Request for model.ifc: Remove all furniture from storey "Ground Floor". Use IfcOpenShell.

First a look at what the model holds.

```python
import ifcopenshell
import ifcopenshell.util.element

model = ifcopenshell.open("model.ifc")
print(model.schema)
storey = next(s for s in model.by_type("IfcBuildingStorey") if s.Name == "Ground Floor")
furniture = [e for e in ifcopenshell.util.element.get_decomposition(storey) if e.is_a("IfcFurnishingElement")]
seen = {}
for e in furniture:
    element_type = ifcopenshell.util.element.get_type(e)
    name = element_type.Name if element_type not in (None, e) else None
    seen[name] = seen.get(name, 0) + 1
for name, count in sorted(seen.items(), key=str):
    print(count, "x", name)
```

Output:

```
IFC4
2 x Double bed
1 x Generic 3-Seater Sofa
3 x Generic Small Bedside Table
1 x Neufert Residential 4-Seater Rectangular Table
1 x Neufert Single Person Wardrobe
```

```python
import ifcopenshell
import ifcopenshell.api.root
import ifcopenshell.util.element

model = ifcopenshell.open("model.ifc")

storey = next(s for s in model.by_type("IfcBuildingStorey") if s.Name == "Ground Floor")
furniture = [e for e in ifcopenshell.util.element.get_decomposition(storey) if e.is_a("IfcFurnishingElement")]

for e in furniture:
    ifcopenshell.api.root.remove_product(model, product=e)
print(len(furniture), "removed")

model.write("model-out.ifc")
```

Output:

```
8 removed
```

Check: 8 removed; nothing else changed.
